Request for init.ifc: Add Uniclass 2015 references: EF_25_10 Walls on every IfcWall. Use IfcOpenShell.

First a look at what the model holds.

```python
import ifcopenshell

model = ifcopenshell.open("init.ifc")
print(model.schema)
print("classifications:", [c.Name for c in model.by_type("IfcClassification")])
for ifc_class in ("IfcDoor", "IfcRoof", "IfcStair", "IfcWall", "IfcWindow"):
    print(ifc_class, len(model.by_type(ifc_class)))
```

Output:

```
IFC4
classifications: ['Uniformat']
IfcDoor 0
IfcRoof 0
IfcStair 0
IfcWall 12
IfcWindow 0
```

```python
import ifcopenshell
import ifcopenshell.api.classification

model = ifcopenshell.open("init.ifc")

system = ifcopenshell.api.classification.add_classification(model, classification="Uniclass 2015")

codes = {
    "IfcWall": ("EF_25_10", "Walls"),
}
for ifc_class, (code, name) in codes.items():
    products = model.by_type(ifc_class)
    ifcopenshell.api.classification.add_reference(
        model, products=products, classification=system, identification=code, name=name
    )
    print(code, len(products))

model.write("init_edited.ifc")
```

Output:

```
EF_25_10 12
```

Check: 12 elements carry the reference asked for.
